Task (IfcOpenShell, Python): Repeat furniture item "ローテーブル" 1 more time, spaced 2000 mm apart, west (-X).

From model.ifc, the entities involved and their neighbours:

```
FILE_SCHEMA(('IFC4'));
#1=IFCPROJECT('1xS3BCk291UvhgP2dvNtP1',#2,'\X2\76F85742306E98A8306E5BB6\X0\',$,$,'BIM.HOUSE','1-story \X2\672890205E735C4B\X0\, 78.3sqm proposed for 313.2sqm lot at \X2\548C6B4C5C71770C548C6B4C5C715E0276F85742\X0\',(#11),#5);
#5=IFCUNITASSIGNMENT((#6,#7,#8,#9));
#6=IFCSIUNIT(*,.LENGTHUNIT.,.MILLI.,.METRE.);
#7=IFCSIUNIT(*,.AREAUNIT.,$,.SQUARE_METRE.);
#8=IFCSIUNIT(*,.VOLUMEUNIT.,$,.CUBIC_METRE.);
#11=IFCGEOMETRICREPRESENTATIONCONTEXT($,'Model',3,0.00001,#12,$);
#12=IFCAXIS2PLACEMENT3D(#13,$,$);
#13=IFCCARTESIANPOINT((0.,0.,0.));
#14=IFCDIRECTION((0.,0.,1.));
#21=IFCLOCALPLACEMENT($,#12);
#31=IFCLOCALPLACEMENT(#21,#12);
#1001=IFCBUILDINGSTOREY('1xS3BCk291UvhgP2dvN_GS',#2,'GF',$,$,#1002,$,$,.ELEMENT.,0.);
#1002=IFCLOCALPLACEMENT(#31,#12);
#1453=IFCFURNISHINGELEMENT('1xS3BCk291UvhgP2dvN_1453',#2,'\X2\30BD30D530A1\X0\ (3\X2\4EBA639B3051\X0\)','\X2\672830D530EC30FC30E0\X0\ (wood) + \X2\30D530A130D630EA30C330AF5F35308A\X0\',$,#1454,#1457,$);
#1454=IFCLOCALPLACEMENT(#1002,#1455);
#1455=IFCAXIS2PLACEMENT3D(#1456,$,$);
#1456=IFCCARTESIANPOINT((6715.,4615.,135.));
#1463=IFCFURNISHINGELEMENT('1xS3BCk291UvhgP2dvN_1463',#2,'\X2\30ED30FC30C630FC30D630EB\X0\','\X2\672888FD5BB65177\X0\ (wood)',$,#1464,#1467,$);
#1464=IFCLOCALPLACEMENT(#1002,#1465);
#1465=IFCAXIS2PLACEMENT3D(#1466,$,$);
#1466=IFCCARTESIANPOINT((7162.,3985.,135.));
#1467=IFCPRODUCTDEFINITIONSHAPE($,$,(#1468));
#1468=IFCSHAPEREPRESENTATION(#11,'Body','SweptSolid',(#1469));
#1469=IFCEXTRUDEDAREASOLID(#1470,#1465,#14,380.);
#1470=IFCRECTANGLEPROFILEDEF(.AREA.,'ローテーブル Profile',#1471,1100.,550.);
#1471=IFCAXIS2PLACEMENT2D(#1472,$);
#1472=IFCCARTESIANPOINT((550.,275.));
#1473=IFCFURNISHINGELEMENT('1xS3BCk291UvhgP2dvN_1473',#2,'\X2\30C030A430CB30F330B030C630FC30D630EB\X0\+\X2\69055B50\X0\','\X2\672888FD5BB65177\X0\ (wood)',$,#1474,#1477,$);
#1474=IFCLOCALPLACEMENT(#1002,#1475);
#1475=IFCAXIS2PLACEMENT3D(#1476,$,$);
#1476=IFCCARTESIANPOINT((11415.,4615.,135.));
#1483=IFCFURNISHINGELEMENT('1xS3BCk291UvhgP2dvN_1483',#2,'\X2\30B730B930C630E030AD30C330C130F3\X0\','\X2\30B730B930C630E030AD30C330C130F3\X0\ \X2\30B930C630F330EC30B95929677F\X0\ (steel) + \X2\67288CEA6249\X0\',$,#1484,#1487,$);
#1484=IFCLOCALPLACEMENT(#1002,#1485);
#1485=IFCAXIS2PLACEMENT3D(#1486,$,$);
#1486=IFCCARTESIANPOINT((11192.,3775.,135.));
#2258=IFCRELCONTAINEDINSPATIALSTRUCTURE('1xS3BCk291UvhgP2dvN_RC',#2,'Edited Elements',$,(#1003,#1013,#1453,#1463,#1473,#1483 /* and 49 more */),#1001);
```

```python
import numpy as np
import ifcopenshell
import ifcopenshell.api.geometry
import ifcopenshell.api.root
import ifcopenshell.util.element
import ifcopenshell.util.placement

model = ifcopenshell.open("model.ifc")


def reuse_history(source, copy):
    """copy_class also copies each property set's owner history, people and application; keep the originals."""
    for rel in copy.IsDefinedBy:
        if rel.is_a("IfcRelDefinesByProperties") and (history := rel.RelatingPropertyDefinition.OwnerHistory):
            rel.RelatingPropertyDefinition.OwnerHistory = source.OwnerHistory
            ifcopenshell.util.element.remove_deep2(model, history)


source = model.by_id(1463)
base = ifcopenshell.util.placement.get_local_placement(source.ObjectPlacement)
step = np.array([-1.0, 0.0, 0.0]) * 2000.0

for i in range(1, 2):
    copy = ifcopenshell.api.root.copy_class(model, product=source)
    copy.Representation = ifcopenshell.util.element.copy_deep(
        model, source.Representation, exclude=["IfcGeometricRepresentationContext", "IfcRepresentationMap"]
    )
    reuse_history(source, copy)
    matrix = base.copy()
    matrix[:3, 3] += i * step
    print("added at", matrix[:3, 3].round(3) + 0.0)
    ifcopenshell.api.geometry.edit_object_placement(model, product=copy, matrix=matrix, is_si=False)

model.write("model_rev.ifc")
```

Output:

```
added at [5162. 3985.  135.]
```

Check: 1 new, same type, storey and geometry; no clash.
